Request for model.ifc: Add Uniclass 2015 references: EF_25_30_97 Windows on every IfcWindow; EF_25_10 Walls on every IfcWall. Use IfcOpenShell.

First a look at what the model holds.

```python
import ifcopenshell

model = ifcopenshell.open("model.ifc")
print(model.schema)
print("classifications:", [c.Name for c in model.by_type("IfcClassification")])
for ifc_class in ("IfcDoor", "IfcRoof", "IfcStair", "IfcWall", "IfcWindow"):
    print(ifc_class, len(model.by_type(ifc_class)))
```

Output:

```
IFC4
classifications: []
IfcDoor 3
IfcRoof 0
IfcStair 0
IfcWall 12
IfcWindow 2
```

```python
import ifcopenshell
import ifcopenshell.api.classification

model = ifcopenshell.open("model.ifc")

system = ifcopenshell.api.classification.add_classification(model, classification="Uniclass 2015")

codes = {
    "IfcWindow": ("EF_25_30_97", "Windows"),
    "IfcWall": ("EF_25_10", "Walls"),
}
for ifc_class, (code, name) in codes.items():
    products = model.by_type(ifc_class)
    ifcopenshell.api.classification.add_reference(
        model, products=products, classification=system, identification=code, name=name
    )
    print(code, len(products))

model.write("model_edited.ifc")
```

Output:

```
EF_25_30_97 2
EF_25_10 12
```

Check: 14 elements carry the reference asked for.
